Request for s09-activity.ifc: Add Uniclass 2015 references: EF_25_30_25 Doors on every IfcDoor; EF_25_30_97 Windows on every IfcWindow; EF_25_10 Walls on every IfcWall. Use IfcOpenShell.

First a look at what the model holds.

```python
import ifcopenshell

model = ifcopenshell.open("s09-activity.ifc")
print(model.schema)
print("classifications:", [c.Name for c in model.by_type("IfcClassification")])
for ifc_class in ("IfcDoor", "IfcRoof", "IfcStair", "IfcWall", "IfcWindow"):
    print(ifc_class, len(model.by_type(ifc_class)))
```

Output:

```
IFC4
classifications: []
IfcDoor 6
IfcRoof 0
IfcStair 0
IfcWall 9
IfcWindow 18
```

```python
import ifcopenshell
import ifcopenshell.api.classification

model = ifcopenshell.open("s09-activity.ifc")

system = ifcopenshell.api.classification.add_classification(model, classification="Uniclass 2015")

codes = {
    "IfcDoor": ("EF_25_30_25", "Doors"),
    "IfcWindow": ("EF_25_30_97", "Windows"),
    "IfcWall": ("EF_25_10", "Walls"),
}
for ifc_class, (code, name) in codes.items():
    products = model.by_type(ifc_class)
    ifcopenshell.api.classification.add_reference(
        model, products=products, classification=system, identification=code, name=name
    )
    print(code, len(products))

model.write("s09-activity_updated.ifc")
```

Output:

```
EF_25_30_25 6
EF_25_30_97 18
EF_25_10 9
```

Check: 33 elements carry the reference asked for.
